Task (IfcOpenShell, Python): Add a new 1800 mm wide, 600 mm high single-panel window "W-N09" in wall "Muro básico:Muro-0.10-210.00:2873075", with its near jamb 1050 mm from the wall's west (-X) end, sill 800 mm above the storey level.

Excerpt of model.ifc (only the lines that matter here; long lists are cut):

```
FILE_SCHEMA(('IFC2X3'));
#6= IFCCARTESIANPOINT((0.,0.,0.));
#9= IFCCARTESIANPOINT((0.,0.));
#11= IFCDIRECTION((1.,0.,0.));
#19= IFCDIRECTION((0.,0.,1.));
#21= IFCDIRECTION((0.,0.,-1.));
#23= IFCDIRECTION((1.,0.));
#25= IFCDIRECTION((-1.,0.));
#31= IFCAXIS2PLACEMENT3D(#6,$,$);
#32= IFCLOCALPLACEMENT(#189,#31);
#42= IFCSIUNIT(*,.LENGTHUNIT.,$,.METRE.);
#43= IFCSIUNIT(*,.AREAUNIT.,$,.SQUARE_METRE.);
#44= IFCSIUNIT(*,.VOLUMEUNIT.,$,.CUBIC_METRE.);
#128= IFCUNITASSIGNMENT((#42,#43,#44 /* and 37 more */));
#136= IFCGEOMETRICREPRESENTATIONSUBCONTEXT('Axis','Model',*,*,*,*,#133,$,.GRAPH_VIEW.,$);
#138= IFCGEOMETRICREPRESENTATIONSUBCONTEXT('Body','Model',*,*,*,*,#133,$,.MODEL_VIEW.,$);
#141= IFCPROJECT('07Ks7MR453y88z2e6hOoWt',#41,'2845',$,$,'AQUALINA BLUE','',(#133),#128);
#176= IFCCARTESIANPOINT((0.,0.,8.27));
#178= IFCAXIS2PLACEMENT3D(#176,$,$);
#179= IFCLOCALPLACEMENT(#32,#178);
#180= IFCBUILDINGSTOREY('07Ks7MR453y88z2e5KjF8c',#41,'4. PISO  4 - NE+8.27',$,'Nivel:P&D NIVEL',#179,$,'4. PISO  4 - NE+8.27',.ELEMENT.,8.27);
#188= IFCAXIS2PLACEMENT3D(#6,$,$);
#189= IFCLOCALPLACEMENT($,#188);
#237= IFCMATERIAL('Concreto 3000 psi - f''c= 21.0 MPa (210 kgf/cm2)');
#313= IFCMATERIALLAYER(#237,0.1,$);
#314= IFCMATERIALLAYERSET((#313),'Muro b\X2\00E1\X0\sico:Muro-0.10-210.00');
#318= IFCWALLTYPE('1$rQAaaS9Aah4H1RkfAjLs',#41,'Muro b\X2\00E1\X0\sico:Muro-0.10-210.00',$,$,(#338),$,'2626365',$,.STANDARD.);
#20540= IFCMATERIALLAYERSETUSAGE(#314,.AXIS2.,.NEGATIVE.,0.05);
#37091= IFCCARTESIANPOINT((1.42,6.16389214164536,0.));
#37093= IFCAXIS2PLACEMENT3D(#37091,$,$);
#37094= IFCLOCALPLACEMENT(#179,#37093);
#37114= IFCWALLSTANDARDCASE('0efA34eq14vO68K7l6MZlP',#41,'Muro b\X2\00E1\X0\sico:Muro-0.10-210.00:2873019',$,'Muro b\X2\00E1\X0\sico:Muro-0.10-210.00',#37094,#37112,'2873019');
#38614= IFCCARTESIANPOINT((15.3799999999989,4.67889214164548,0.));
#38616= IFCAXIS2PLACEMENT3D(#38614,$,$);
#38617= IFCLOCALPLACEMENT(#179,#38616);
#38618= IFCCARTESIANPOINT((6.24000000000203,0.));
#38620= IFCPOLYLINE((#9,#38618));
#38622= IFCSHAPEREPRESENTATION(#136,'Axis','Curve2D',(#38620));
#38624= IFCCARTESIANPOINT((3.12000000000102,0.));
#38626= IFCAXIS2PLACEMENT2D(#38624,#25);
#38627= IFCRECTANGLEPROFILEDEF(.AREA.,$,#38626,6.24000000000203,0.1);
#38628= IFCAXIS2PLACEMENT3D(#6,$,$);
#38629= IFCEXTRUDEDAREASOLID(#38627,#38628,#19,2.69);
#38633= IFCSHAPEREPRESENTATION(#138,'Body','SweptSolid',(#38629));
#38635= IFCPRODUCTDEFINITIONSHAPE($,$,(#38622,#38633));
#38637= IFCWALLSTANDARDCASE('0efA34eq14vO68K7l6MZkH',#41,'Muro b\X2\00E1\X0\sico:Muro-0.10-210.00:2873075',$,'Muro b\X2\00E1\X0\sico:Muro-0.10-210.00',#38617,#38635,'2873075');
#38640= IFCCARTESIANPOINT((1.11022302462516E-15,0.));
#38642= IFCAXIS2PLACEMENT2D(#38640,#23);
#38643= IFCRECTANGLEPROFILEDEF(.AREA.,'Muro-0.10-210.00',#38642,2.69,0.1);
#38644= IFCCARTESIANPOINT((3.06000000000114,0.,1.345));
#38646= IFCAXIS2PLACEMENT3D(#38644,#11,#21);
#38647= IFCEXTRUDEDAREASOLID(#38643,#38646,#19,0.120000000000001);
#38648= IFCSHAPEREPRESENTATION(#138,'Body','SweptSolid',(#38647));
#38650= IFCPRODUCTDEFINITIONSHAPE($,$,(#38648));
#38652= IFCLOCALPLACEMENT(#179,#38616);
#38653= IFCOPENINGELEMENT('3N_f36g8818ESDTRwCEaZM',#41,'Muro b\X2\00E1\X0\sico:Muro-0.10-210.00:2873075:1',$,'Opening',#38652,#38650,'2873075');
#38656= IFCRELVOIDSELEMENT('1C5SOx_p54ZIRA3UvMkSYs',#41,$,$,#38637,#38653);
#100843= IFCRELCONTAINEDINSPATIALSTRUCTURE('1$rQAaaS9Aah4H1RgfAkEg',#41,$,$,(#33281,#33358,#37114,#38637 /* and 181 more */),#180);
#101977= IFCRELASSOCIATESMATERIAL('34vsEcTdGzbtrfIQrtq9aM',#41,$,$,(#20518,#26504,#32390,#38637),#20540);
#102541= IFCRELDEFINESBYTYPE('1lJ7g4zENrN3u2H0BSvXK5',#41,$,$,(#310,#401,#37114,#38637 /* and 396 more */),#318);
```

```python
import numpy as np
import ifcopenshell
import ifcopenshell.api.feature
import ifcopenshell.api.geometry
import ifcopenshell.api.root
import ifcopenshell.api.spatial
import ifcopenshell.api.type
import ifcopenshell.geom
import ifcopenshell.util.element
import ifcopenshell.util.placement
import ifcopenshell.util.representation
import ifcopenshell.util.shape
import ifcopenshell.util.unit

model = ifcopenshell.open("model.ifc")
unit_scale = ifcopenshell.util.unit.calculate_unit_scale(model)
settings = ifcopenshell.geom.settings()


def volume(element):
    """Net volume in cubic metres, openings subtracted."""
    shape = ifcopenshell.geom.create_shape(settings, element)
    return ifcopenshell.util.shape.get_volume(shape.geometry)


wall = model.by_id(38637)
storey = ifcopenshell.util.element.get_container(wall, ifc_class="IfcBuildingStorey")
context = ifcopenshell.util.representation.get_context(model, "Model", "Body", "MODEL_VIEW")
before = volume(wall)

width, height, from_end, sill = 1.8, 0.6, 1.05, 0.8  # metres

# The wall runs along its own X axis, and the end named is its -X end.
wall_shape = ifcopenshell.geom.create_shape(settings, wall)
x, y, z = ifcopenshell.util.shape.get_vertices(wall_shape.geometry).T
start = x.min() + from_end
face, thickness = float(y.min()), float(y.max() - y.min())
wall_matrix = ifcopenshell.util.placement.get_local_placement(wall.ObjectPlacement)
level = ifcopenshell.util.placement.get_local_placement(storey.ObjectPlacement)[2, 3]


def in_wall(x, y):
    """Placement at x, y metres in the wall's axes, at sill height."""
    matrix = wall_matrix.copy()
    matrix[:, 3] = wall_matrix @ np.array([x / unit_scale, y / unit_scale, 0.0, 1.0])
    matrix[2, 3] = level + sill / unit_scale
    return matrix


# Opening: a box that overshoots both wall faces by 50 mm.
opening = ifcopenshell.api.root.create_entity(model, ifc_class="IfcOpeningElement")
box = ifcopenshell.api.geometry.add_wall_representation(
    model, context=context, length=width, height=height, thickness=thickness + 0.1
)
ifcopenshell.api.geometry.assign_representation(model, product=opening, representation=box)
ifcopenshell.api.geometry.edit_object_placement(model, product=opening, matrix=in_wall(start, face - 0.05), is_si=False)
ifcopenshell.api.feature.add_feature(model, feature=opening, element=wall)

window = ifcopenshell.api.root.create_entity(model, ifc_class="IfcWindow", name="W-N09")
window.OverallWidth, window.OverallHeight = width / unit_scale, height / unit_scale
body = ifcopenshell.api.geometry.add_window_representation(
    model,
    context=context,
    overall_width=window.OverallWidth,
    overall_height=window.OverallHeight,
    partition_type="SINGLE_PANEL",
)
ifcopenshell.api.geometry.assign_representation(model, product=window, representation=body)
ifcopenshell.api.spatial.assign_container(model, products=[window], relating_structure=storey)
fills = ifcopenshell.api.feature.add_filling(model, opening=opening, element=window)
fills.OwnerHistory = window.OwnerHistory  # required in IFC2X3

# IFC2X3 keeps the operation on the window style.
style = ifcopenshell.api.root.create_entity(model, ifc_class="IfcWindowStyle", name="W-N09")
style.OperationType, style.ConstructionType = "SINGLE_PANEL", "NOTDEFINED"
style.ParameterTakesPrecedence = style.Sizeable = False
ifcopenshell.api.type.assign_type(model, related_objects=[window], relating_type=style)

# Centre the window in the wall's thickness.
ifcopenshell.api.geometry.edit_object_placement(model, product=window, matrix=in_wall(start, face), is_si=False)
window_shape = ifcopenshell.geom.create_shape(settings, window)
depth = ifcopenshell.util.shape.get_vertices(window_shape.geometry)[:, 1]
offset = face + thickness / 2 - (depth.min() + depth.max()) / 2
ifcopenshell.api.geometry.edit_object_placement(model, product=window, matrix=in_wall(start, offset), is_si=False)

after = volume(wall)

print(f"wall volume {before:.3f} -> {after:.3f} m3")

model.write("model-out.ifc")
```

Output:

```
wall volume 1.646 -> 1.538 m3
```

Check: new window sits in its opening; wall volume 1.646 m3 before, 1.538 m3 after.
